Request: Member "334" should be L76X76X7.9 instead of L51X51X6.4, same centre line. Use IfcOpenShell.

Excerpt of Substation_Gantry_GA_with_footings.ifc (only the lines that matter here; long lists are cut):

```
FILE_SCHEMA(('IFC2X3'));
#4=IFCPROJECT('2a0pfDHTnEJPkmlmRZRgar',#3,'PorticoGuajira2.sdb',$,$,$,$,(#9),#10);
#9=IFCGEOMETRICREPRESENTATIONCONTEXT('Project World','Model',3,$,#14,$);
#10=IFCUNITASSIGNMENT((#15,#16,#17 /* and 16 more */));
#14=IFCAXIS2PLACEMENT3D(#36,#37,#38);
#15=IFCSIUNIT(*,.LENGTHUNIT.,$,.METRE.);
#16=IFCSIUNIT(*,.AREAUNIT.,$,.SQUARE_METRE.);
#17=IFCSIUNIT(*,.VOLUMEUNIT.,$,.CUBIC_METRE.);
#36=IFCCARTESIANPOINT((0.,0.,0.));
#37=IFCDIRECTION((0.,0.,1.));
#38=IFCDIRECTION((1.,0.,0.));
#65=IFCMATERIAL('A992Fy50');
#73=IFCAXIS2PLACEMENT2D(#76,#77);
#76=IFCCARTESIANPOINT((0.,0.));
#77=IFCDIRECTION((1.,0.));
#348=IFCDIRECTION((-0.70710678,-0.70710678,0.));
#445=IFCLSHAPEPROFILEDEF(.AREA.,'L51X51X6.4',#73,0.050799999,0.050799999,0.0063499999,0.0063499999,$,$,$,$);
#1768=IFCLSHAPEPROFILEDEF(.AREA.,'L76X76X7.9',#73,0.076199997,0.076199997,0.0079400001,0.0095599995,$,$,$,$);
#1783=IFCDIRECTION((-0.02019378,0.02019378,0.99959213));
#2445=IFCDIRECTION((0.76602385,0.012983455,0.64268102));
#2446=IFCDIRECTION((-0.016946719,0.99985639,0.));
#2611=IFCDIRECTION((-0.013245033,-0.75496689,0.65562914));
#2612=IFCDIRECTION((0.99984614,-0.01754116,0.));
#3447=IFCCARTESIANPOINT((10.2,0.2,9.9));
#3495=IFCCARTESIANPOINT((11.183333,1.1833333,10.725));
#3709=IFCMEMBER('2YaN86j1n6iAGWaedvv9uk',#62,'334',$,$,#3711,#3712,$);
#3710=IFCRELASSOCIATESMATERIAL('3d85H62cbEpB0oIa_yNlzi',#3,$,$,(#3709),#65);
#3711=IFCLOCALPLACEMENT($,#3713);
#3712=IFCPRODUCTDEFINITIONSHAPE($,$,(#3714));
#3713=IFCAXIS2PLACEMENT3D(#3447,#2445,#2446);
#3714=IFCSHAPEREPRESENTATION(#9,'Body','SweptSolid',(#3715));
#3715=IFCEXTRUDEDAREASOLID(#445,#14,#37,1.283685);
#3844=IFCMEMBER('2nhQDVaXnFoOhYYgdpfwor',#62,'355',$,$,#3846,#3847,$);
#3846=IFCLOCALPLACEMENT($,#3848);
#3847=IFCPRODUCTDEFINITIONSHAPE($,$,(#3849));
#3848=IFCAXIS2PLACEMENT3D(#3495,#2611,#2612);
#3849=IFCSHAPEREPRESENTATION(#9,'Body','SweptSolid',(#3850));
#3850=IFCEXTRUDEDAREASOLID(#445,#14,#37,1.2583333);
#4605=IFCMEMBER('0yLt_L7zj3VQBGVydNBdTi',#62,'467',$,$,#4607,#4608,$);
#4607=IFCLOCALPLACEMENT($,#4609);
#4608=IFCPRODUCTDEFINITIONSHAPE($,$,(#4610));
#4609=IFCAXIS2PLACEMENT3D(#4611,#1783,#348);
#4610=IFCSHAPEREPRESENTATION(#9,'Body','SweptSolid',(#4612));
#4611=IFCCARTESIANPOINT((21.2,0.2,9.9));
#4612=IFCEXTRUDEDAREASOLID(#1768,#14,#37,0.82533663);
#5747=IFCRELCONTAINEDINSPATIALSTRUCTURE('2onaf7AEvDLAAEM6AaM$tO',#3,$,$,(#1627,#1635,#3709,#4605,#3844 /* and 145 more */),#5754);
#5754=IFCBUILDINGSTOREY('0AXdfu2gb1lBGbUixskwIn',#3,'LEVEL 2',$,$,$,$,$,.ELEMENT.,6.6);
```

```python
import ifcopenshell
import ifcopenshell.util.element

model = ifcopenshell.open("Substation_Gantry_GA_with_footings.ifc")

member = model.by_guid("2YaN86j1n6iAGWaedvv9uk")
source = next(p for p in model.by_type("IfcLShapeProfileDef") if p.ProfileName == "L76X76X7.9")

body = next(r for r in member.Representation.Representations if r.RepresentationIdentifier == "Body")
solid = body.Items[0]
old_profile = solid.SweptArea

# Copy the section's sizes but keep this member's own profile position.
profile = ifcopenshell.util.element.copy(model, source)
profile.Position = old_profile.Position
solid.SweptArea = profile
if not model.get_total_inverses(old_profile):
    ifcopenshell.util.element.remove_deep2(model, old_profile)

print(solid.SweptArea)

model.write("Substation_Gantry_GA_with_footings_rev.ifc")
```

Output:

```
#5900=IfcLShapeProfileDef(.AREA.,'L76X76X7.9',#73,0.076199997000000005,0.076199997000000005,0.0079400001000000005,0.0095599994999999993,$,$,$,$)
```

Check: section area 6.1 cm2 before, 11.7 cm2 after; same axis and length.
